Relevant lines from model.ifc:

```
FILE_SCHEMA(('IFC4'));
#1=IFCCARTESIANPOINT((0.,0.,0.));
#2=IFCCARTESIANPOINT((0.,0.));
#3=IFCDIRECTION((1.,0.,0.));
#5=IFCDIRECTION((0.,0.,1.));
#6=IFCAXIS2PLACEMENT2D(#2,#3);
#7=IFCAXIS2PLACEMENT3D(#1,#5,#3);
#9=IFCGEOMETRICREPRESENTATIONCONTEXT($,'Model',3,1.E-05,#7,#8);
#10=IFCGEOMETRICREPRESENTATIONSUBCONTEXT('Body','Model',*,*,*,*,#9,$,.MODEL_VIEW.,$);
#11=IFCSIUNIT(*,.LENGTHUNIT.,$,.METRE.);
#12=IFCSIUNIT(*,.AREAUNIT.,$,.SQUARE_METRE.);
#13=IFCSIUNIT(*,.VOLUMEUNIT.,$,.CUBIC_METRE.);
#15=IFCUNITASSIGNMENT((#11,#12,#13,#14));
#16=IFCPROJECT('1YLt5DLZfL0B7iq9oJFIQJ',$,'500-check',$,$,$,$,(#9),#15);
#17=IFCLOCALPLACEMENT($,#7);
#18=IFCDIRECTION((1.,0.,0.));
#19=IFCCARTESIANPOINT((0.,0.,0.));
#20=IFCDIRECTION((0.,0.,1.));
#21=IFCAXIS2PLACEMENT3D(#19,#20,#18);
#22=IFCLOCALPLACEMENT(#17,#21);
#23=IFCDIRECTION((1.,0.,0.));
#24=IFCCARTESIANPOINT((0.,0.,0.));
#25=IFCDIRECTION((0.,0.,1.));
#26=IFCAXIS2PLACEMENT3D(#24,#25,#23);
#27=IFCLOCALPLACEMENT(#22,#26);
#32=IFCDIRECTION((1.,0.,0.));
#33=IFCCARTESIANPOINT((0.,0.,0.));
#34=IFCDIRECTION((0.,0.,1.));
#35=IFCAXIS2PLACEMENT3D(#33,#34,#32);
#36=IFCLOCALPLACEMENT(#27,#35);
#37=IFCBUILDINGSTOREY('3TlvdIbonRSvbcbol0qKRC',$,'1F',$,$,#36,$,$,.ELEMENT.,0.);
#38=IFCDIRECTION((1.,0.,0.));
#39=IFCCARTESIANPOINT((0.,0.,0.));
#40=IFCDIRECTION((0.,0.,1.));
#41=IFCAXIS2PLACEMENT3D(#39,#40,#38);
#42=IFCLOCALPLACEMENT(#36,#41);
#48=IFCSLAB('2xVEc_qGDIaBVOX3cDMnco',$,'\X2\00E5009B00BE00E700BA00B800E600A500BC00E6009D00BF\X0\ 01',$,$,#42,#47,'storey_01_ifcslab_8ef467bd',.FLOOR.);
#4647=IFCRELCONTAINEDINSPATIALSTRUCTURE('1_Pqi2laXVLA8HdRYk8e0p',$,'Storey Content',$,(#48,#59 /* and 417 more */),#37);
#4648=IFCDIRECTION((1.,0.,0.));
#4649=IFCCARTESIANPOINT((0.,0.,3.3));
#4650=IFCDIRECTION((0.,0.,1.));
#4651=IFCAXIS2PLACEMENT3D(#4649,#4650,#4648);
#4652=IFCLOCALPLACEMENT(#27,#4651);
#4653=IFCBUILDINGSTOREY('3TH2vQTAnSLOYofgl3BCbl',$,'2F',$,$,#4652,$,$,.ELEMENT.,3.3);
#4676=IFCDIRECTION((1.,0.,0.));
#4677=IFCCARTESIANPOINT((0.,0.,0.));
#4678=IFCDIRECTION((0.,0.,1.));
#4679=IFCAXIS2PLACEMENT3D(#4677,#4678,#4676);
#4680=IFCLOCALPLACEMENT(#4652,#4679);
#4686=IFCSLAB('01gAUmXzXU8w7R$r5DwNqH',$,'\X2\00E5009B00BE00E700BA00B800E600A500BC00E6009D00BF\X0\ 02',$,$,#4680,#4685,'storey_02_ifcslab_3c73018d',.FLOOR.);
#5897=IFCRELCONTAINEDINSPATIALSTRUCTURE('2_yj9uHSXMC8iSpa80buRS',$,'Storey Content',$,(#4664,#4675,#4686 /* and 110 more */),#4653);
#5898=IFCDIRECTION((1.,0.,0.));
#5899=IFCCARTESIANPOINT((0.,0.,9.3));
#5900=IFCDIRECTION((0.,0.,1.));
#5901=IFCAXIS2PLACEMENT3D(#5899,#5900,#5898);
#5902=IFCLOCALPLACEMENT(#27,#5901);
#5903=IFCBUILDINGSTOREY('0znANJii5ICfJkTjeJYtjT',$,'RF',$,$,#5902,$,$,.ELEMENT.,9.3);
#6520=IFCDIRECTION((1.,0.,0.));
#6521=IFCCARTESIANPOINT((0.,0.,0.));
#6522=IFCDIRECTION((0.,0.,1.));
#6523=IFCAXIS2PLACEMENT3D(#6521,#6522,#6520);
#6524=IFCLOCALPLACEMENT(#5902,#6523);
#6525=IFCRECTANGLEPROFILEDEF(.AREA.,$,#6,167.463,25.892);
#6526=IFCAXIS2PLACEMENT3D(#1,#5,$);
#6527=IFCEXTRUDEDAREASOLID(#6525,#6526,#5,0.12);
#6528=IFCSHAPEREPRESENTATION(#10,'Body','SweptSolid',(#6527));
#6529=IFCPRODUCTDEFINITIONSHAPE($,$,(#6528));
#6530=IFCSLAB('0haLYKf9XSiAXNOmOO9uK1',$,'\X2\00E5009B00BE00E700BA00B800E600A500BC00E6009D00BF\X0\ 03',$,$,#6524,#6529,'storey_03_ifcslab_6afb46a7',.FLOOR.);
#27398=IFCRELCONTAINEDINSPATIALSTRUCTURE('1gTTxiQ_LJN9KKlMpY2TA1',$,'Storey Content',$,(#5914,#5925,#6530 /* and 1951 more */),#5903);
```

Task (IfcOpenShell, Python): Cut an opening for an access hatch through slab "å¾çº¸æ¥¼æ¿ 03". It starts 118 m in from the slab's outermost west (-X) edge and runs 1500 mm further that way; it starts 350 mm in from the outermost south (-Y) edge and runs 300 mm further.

```python
import numpy as np
import ifcopenshell
import ifcopenshell.api.feature
import ifcopenshell.api.geometry
import ifcopenshell.api.root
import ifcopenshell.geom
import ifcopenshell.util.placement
import ifcopenshell.util.representation
import ifcopenshell.util.shape
import ifcopenshell.util.unit

model = ifcopenshell.open("model.ifc")
unit_scale = ifcopenshell.util.unit.calculate_unit_scale(model)
settings = ifcopenshell.geom.settings()


def volume(element):
    """Net volume in cubic metres, openings subtracted."""
    shape = ifcopenshell.geom.create_shape(settings, element)
    return ifcopenshell.util.shape.get_volume(shape.geometry)


slab = model.by_guid("0haLYKf9XSiAXNOmOO9uK1")
before = volume(slab)

# Extent in the slab's own axes, in metres. The edges named are its -X and -Y sides.
slab_shape = ifcopenshell.geom.create_shape(settings, slab)
vertices = ifcopenshell.util.shape.get_vertices(slab_shape.geometry)
x_min, y_min, bottom = vertices.min(axis=0)
top = vertices[:, 2].max()

opening = ifcopenshell.api.root.create_entity(model, ifc_class="IfcOpeningElement", name="Access hatch opening", predefined_type="OPENING")
context = ifcopenshell.util.representation.get_context(model, "Model", "Body", "MODEL_VIEW")
width, depth = 1.5, 0.3
outline = [(0.0, 0.0), (width, 0.0), (width, depth), (0.0, depth), (0.0, 0.0)]
# Overshoot both faces by 50 mm so the cut is clean.
shape = ifcopenshell.api.geometry.add_slab_representation(
    model, context=context, depth=top - bottom + 0.1, polyline=outline
)
ifcopenshell.api.geometry.assign_representation(model, product=opening, representation=shape)

matrix = ifcopenshell.util.placement.get_local_placement(slab.ObjectPlacement)
matrix[:, 3] = matrix @ np.append(np.array([x_min + 118, y_min + 0.35, bottom - 0.05]) / unit_scale, 1.0)
ifcopenshell.api.geometry.edit_object_placement(model, product=opening, matrix=matrix, is_si=False)
ifcopenshell.api.feature.add_feature(model, feature=opening, element=slab)

after = volume(slab)

print(f"slab volume {before:.3f} -> {after:.3f} m3")

model.write("model_edited.ifc")
```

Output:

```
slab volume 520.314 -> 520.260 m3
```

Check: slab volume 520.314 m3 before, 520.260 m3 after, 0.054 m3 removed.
